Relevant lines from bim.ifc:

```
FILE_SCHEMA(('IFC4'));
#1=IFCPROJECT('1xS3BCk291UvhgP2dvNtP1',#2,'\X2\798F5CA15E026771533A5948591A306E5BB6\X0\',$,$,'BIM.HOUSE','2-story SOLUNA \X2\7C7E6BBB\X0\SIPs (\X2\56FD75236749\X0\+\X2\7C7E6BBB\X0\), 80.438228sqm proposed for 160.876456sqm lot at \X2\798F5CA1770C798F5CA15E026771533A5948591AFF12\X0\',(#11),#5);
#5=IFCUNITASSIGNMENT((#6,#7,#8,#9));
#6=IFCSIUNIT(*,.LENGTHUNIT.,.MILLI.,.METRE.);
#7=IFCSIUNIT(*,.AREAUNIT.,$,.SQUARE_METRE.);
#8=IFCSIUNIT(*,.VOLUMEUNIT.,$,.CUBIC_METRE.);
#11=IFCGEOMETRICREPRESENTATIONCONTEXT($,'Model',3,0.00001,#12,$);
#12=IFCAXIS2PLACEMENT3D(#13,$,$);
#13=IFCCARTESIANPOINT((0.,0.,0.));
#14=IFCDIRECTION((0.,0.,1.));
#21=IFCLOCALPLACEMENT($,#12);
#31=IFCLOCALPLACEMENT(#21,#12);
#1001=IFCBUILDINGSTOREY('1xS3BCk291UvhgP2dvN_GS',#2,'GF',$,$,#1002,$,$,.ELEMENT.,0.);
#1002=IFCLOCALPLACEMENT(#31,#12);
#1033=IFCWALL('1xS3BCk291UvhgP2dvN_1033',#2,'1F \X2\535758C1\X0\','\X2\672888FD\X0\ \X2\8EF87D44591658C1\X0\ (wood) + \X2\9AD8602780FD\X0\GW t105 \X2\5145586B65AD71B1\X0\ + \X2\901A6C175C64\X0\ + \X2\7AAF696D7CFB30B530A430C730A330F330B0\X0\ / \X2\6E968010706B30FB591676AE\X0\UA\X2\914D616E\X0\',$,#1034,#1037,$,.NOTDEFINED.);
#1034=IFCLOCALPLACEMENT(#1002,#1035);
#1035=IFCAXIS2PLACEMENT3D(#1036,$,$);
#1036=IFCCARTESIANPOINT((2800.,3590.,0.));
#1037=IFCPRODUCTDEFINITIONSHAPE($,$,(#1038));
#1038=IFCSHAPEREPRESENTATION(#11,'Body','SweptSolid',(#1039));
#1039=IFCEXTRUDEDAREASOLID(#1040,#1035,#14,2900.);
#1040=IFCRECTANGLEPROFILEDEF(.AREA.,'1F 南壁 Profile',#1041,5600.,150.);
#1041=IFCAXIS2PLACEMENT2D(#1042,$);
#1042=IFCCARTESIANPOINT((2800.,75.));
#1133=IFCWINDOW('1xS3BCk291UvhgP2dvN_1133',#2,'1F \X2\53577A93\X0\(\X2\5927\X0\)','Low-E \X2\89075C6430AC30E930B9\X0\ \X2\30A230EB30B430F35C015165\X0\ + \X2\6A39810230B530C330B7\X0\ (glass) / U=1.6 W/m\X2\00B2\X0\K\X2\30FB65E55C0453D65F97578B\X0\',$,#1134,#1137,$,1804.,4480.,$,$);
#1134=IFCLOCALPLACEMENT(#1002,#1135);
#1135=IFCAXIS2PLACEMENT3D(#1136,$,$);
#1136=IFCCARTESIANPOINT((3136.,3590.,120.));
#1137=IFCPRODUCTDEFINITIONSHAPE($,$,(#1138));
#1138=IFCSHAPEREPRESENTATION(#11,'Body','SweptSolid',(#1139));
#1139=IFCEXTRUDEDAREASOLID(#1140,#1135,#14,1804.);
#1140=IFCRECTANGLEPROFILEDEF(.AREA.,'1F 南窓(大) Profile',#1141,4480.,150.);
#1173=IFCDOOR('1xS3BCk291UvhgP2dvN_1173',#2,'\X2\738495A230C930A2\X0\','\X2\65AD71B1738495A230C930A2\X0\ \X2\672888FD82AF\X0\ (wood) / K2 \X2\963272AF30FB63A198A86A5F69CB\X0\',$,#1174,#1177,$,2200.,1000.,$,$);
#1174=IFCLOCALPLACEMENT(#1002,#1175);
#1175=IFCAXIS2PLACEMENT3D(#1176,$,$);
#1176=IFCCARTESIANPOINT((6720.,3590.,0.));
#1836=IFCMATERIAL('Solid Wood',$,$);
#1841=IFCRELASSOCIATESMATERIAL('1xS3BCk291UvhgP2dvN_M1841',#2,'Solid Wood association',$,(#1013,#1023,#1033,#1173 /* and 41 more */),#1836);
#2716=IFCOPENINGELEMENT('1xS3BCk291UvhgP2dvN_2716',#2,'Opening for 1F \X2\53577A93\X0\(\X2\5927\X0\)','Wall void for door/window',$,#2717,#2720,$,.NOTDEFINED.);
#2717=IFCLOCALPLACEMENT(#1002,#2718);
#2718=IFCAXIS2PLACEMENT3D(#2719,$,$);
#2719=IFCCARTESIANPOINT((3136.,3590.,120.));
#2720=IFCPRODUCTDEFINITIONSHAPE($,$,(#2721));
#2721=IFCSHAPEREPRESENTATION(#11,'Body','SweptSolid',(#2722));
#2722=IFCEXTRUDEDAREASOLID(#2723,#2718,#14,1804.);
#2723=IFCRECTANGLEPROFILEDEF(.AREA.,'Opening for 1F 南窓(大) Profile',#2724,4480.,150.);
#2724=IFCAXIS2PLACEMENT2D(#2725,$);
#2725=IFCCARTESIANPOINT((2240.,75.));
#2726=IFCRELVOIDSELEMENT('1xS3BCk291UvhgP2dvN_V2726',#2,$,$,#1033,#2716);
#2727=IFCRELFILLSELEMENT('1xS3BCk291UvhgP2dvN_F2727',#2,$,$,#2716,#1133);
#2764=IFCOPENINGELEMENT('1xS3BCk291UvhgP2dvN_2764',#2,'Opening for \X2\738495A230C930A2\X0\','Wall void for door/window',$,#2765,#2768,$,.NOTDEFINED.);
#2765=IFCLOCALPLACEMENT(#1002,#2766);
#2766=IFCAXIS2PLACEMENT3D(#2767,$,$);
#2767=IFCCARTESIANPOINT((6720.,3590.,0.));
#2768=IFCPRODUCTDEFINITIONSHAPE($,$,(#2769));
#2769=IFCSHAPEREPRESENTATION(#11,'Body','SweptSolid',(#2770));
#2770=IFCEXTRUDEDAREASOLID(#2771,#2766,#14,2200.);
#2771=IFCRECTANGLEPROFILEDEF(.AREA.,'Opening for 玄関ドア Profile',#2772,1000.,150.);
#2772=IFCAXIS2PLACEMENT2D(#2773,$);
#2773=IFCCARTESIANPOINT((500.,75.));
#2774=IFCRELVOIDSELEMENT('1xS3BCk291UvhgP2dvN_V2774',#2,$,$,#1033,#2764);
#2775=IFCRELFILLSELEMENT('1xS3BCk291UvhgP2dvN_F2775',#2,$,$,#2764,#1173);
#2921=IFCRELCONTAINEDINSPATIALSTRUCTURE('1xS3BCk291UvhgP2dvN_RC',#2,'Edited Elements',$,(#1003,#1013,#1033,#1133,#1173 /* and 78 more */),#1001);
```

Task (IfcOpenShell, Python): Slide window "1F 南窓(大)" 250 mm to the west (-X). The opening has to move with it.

```python
import ifcopenshell
import ifcopenshell.api.geometry
import ifcopenshell.util.placement
import ifcopenshell.util.unit

model = ifcopenshell.open("bim.ifc")
unit_scale = ifcopenshell.util.unit.calculate_unit_scale(model)

window = model.by_guid("1xS3BCk291UvhgP2dvN_1133")
opening = window.FillsVoids[0].RelatingOpeningElement
wall = opening.VoidsElements[0].RelatingBuildingElement

wall_matrix = ifcopenshell.util.placement.get_local_placement(wall.ObjectPlacement)
shift = wall_matrix[:3, 0] * -0.25 / unit_scale
before = ifcopenshell.util.placement.get_local_placement(window.ObjectPlacement)[:3, 3].copy()

# The window is not placed relative to its opening, so move both.
for product in (opening, window):
    matrix = ifcopenshell.util.placement.get_local_placement(product.ObjectPlacement)
    matrix[:3, 3] += shift
    ifcopenshell.api.geometry.edit_object_placement(model, product=product, matrix=matrix, is_si=False)

after = ifcopenshell.util.placement.get_local_placement(window.ObjectPlacement)[:3, 3]
print("window moved by", (after - before).round(3) + 0.0)

model.write("bim-out.ifc")
```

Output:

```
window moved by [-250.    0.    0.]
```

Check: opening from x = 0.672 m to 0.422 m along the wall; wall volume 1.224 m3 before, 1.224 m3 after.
